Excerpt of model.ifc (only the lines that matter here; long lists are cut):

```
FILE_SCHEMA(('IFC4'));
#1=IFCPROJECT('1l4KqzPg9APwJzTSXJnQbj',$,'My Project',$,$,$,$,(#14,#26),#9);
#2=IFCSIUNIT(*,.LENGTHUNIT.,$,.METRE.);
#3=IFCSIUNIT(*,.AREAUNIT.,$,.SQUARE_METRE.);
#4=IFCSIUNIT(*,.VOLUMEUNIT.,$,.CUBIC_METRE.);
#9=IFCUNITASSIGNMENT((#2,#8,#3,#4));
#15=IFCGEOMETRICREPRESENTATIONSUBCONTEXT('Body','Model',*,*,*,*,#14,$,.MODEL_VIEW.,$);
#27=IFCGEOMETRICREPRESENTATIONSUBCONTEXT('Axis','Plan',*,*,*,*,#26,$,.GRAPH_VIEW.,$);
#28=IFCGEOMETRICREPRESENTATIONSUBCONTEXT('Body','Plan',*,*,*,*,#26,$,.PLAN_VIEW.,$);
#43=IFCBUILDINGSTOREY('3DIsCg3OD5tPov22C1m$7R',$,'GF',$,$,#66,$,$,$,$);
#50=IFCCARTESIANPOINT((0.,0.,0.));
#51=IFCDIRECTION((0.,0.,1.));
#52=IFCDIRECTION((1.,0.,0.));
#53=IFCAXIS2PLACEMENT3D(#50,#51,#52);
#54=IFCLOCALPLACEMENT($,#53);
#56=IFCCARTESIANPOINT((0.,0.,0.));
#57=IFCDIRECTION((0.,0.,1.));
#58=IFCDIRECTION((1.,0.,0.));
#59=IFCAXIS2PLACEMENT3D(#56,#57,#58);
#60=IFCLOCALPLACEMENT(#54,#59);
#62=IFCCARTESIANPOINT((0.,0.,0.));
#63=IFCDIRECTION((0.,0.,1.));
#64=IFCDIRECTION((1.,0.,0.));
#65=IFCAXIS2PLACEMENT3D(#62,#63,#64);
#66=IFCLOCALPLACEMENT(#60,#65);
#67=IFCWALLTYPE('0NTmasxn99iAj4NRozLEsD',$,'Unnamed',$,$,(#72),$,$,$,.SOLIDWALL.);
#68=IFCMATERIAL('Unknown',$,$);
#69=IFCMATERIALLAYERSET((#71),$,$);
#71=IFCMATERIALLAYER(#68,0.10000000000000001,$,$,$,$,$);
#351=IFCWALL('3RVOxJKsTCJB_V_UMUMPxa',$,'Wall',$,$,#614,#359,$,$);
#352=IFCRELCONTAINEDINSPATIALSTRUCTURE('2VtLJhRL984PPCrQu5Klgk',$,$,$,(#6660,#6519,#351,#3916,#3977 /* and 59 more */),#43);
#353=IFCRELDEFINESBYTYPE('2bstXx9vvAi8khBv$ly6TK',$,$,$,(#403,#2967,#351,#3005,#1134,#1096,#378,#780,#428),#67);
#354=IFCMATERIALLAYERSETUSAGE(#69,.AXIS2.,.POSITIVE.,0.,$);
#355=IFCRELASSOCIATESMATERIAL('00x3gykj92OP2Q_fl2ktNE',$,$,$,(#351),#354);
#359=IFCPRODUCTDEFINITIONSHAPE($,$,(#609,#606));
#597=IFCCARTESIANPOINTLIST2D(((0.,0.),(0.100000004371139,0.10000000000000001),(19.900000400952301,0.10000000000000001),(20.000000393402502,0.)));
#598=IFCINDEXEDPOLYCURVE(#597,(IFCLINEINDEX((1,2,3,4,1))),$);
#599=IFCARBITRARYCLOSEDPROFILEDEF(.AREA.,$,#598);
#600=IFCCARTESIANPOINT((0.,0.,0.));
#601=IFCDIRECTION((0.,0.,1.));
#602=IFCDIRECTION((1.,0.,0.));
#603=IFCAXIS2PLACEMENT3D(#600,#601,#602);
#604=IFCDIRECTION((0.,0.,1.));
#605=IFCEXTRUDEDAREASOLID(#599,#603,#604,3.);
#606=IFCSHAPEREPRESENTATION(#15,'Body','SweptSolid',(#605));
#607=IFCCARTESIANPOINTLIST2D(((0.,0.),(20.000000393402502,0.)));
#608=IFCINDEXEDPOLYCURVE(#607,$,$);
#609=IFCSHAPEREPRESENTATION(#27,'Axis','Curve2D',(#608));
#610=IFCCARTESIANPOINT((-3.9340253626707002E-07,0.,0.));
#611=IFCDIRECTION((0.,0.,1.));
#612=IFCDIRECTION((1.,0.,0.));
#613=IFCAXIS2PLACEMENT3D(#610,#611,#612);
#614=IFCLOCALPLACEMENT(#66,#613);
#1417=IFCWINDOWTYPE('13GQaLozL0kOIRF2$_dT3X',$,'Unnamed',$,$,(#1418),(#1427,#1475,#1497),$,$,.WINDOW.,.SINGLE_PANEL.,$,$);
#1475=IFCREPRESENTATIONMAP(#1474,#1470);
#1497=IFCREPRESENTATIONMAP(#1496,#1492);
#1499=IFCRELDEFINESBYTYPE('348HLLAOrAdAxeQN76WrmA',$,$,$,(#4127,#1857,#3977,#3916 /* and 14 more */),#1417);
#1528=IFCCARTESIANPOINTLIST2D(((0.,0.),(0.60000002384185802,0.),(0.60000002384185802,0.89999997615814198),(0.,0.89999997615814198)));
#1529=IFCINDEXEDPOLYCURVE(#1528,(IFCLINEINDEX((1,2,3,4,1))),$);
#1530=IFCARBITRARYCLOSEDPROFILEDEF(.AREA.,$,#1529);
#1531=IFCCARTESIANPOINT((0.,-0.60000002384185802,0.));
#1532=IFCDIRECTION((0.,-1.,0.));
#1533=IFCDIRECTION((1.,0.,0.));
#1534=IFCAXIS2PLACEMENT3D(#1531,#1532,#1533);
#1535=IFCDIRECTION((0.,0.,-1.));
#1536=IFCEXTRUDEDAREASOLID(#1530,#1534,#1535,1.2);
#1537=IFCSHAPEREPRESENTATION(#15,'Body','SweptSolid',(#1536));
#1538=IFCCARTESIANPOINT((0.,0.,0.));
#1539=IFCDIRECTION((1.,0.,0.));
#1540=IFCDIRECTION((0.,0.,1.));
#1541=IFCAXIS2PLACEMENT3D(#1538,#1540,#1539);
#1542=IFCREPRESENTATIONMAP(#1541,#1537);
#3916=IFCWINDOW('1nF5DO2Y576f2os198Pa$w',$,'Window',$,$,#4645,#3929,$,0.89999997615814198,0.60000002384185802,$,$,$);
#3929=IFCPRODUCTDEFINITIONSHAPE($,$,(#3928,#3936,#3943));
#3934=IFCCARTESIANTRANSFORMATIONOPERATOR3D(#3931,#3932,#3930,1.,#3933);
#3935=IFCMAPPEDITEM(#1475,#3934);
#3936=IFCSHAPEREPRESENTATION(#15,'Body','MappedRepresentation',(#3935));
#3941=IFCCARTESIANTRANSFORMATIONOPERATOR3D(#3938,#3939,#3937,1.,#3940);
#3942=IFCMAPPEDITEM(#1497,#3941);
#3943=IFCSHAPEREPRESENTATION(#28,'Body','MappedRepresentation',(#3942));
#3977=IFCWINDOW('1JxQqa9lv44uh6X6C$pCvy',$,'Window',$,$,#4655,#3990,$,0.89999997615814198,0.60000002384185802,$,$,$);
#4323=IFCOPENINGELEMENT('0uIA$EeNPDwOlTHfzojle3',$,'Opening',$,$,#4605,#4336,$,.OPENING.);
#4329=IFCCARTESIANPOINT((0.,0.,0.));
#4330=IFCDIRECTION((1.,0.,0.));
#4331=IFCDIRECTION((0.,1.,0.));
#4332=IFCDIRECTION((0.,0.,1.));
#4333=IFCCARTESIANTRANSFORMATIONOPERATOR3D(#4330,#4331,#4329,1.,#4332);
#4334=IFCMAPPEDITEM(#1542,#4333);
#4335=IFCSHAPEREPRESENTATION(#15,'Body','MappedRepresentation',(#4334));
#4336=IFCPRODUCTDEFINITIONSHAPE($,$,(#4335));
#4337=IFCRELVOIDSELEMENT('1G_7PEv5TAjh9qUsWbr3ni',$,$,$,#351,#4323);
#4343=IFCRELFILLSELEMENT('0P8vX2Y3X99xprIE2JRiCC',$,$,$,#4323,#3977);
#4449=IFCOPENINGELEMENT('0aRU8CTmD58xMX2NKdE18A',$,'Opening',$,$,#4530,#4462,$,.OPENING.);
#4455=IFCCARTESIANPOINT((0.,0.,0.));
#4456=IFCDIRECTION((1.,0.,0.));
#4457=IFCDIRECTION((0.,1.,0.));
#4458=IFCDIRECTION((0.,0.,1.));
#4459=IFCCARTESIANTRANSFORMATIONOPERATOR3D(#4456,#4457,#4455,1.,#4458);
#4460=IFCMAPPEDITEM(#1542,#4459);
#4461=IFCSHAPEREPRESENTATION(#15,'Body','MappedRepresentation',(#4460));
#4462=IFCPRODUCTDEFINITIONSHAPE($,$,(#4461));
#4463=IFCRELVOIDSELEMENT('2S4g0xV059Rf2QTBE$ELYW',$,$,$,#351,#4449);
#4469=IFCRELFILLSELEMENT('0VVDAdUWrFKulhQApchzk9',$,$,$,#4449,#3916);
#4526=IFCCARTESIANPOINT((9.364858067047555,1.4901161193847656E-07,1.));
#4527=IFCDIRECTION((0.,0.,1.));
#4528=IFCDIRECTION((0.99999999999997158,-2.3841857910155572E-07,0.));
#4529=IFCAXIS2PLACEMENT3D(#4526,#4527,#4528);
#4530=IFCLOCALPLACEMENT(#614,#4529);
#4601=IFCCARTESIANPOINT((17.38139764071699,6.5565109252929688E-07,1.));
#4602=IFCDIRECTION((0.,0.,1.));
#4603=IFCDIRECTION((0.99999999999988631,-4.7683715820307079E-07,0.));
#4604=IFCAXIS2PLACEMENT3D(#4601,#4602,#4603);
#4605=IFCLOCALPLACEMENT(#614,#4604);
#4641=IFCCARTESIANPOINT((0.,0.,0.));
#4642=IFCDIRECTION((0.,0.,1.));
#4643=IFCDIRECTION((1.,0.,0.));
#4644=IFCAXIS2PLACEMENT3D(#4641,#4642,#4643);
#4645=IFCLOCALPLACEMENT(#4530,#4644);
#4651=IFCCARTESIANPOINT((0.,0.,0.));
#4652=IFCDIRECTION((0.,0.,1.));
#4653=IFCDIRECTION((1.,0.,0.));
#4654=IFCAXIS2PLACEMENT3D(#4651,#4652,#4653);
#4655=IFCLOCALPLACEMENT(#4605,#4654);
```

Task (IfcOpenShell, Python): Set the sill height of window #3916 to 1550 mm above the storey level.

```python
import numpy as np
import ifcopenshell
import ifcopenshell.api.geometry
import ifcopenshell.geom
import ifcopenshell.util.element
import ifcopenshell.util.placement
import ifcopenshell.util.shape
import ifcopenshell.util.unit

model = ifcopenshell.open("model.ifc")
unit_scale = ifcopenshell.util.unit.calculate_unit_scale(model)

window = model.by_guid("1nF5DO2Y576f2os198Pa$w")
opening = window.FillsVoids[0].RelatingOpeningElement
storey = ifcopenshell.util.element.get_container(window, ifc_class="IfcBuildingStorey")
level = ifcopenshell.util.placement.get_local_placement(storey.ObjectPlacement)[2, 3]

# The opening's origin need not be at the sill, so measure its lowest point.
shape = ifcopenshell.geom.create_shape(ifcopenshell.geom.settings(), opening)
bottom = ifcopenshell.util.shape.get_shape_bottom_elevation(shape, shape.geometry) / unit_scale
dz = level + 1.55 / unit_scale - bottom

shift = np.array([0.0, 0.0, dz])
# The window is placed relative to its opening, so it follows when the opening moves.
matrix = ifcopenshell.util.placement.get_local_placement(opening.ObjectPlacement)
matrix[:3, 3] += shift
ifcopenshell.api.geometry.edit_object_placement(
    model, product=opening, matrix=matrix, is_si=False, should_transform_children=True
)

print(f"moved by {dz * unit_scale:+.3f} m")

model.write("model_rev.ifc")
```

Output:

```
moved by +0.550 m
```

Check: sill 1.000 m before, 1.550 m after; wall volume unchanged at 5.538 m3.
